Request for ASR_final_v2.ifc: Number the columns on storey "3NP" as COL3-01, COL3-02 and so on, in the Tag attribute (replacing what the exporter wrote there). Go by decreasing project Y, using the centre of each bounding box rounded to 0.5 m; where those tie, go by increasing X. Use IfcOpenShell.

First a look at what the model holds.

```python
import ifcopenshell
import ifcopenshell.util.element
import ifcopenshell.util.placement

model = ifcopenshell.open("ASR_final_v2.ifc")
print(model.schema)
storey = next(s for s in model.by_type("IfcBuildingStorey") if s.Name == "3NP")
columns = [e for e in ifcopenshell.util.element.get_decomposition(storey) if e.is_a("IfcColumn")]
for e in sorted(columns, key=lambda e: e.id()):
    origin = ifcopenshell.util.placement.get_local_placement(e.ObjectPlacement)[:3, 3]
    print(e.id(), e.Tag, e.Name, origin.round(2) + 0.0, sep=" | ")
```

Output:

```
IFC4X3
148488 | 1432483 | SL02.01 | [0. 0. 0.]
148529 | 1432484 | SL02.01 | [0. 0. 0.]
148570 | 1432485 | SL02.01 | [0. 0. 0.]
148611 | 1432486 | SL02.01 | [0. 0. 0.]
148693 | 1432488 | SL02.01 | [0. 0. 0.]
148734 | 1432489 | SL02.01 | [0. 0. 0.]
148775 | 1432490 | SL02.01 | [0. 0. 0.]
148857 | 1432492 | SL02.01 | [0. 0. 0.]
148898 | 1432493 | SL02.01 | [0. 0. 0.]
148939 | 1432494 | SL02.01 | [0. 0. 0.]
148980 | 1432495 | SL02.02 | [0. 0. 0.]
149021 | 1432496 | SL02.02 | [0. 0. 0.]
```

```python
import ifcopenshell
import ifcopenshell.geom
import ifcopenshell.util.element
import ifcopenshell.util.shape

model = ifcopenshell.open("ASR_final_v2.ifc")
settings = ifcopenshell.geom.settings()
settings.set("use-world-coords", True)


def centre(element):
    shape = ifcopenshell.geom.create_shape(settings, element)
    return ifcopenshell.util.shape.get_bbox_centroid(shape.geometry)


storey = next(s for s in model.by_type("IfcBuildingStorey") if s.Name == "3NP")
columns = [e for e in ifcopenshell.util.element.get_decomposition(storey) if e.is_a("IfcColumn")]

# Insertion points can sit at a corner or the storey origin, so sort by the geometry (in metres).
centres = {e: centre(e) for e in columns}
columns.sort(key=lambda e: (-round(centres[e][1] / 0.5), centres[e][0]))

for i, e in enumerate(columns, start=1):
    number = f"COL3-{i:02d}"
    e.Tag = number
    print(e.id(), number)

model.write("ASR_final_v2-out.ifc")
```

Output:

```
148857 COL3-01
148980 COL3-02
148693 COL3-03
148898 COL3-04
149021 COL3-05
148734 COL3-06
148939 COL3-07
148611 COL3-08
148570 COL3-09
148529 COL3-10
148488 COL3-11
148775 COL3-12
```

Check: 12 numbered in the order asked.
